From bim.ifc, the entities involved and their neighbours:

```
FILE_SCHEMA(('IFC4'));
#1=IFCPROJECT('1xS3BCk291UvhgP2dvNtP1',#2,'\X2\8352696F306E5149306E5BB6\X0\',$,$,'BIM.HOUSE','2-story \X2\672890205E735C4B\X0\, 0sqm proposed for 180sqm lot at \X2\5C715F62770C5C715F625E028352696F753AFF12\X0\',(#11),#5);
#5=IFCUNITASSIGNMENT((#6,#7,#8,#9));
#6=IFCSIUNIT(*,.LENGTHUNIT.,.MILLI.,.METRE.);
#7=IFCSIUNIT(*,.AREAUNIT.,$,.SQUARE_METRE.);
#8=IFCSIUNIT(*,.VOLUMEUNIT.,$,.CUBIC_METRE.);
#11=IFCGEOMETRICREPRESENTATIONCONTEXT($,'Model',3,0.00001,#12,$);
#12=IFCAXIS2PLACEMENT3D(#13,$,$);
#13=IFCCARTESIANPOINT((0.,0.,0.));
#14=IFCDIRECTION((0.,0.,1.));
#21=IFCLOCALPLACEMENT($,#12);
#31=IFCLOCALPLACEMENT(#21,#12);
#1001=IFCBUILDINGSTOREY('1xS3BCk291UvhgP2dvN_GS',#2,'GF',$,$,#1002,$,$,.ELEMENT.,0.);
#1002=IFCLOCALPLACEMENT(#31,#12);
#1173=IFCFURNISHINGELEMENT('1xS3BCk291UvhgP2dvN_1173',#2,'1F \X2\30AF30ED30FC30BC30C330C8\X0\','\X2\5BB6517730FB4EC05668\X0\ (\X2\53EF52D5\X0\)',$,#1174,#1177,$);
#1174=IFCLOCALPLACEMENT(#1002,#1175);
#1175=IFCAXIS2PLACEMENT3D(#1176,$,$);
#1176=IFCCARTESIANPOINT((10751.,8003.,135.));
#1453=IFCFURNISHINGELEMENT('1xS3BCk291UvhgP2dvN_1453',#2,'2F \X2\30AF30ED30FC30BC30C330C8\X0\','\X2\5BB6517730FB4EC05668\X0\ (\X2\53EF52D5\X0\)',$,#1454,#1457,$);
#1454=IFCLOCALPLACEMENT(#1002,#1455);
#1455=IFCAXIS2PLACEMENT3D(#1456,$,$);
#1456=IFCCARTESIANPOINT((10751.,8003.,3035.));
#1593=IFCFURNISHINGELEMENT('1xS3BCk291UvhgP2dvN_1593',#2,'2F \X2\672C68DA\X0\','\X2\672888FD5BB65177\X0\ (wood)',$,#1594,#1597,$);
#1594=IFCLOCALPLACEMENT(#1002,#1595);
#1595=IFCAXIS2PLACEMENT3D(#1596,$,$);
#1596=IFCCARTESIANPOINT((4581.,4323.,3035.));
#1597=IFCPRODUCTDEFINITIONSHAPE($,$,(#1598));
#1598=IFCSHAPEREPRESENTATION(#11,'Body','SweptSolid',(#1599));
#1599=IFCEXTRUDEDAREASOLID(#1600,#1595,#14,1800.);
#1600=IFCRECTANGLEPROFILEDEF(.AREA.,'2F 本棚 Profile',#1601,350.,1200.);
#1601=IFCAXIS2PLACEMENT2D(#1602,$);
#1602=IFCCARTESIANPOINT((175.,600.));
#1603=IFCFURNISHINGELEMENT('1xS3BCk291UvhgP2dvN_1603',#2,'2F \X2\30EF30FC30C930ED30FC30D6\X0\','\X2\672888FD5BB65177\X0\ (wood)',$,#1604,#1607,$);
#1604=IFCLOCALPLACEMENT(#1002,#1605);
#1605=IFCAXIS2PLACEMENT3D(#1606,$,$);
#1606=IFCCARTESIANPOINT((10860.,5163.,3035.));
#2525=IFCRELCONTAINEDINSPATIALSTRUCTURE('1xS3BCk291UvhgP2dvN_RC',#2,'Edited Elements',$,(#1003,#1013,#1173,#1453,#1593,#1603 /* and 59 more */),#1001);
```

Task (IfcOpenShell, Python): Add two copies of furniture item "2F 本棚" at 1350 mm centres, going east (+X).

```python
import numpy as np
import ifcopenshell
import ifcopenshell.api.geometry
import ifcopenshell.api.root
import ifcopenshell.util.element
import ifcopenshell.util.placement
import ifcopenshell.util.unit

model = ifcopenshell.open("bim.ifc")
unit_scale = ifcopenshell.util.unit.calculate_unit_scale(model)


def reuse_history(source, copy):
    """copy_class also copies each property set's owner history, people and application; keep the originals."""
    for rel in copy.IsDefinedBy:
        if rel.is_a("IfcRelDefinesByProperties") and (history := rel.RelatingPropertyDefinition.OwnerHistory):
            rel.RelatingPropertyDefinition.OwnerHistory = source.OwnerHistory
            ifcopenshell.util.element.remove_deep2(model, history)


source = model.by_guid("1xS3BCk291UvhgP2dvN_1593")
base = ifcopenshell.util.placement.get_local_placement(source.ObjectPlacement)
step = np.array([1.0, 0.0, 0.0]) * 1.35 / unit_scale

for i in range(1, 3):
    copy = ifcopenshell.api.root.copy_class(model, product=source)
    copy.Representation = ifcopenshell.util.element.copy_deep(
        model, source.Representation, exclude=["IfcGeometricRepresentationContext", "IfcRepresentationMap"]
    )
    reuse_history(source, copy)
    matrix = base.copy()
    matrix[:3, 3] += i * step
    print("added at", matrix[:3, 3].round(3) + 0.0)
    ifcopenshell.api.geometry.edit_object_placement(model, product=copy, matrix=matrix, is_si=False)

model.write("bim_edited.ifc")
```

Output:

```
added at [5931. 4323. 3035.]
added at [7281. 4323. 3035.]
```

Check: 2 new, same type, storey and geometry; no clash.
